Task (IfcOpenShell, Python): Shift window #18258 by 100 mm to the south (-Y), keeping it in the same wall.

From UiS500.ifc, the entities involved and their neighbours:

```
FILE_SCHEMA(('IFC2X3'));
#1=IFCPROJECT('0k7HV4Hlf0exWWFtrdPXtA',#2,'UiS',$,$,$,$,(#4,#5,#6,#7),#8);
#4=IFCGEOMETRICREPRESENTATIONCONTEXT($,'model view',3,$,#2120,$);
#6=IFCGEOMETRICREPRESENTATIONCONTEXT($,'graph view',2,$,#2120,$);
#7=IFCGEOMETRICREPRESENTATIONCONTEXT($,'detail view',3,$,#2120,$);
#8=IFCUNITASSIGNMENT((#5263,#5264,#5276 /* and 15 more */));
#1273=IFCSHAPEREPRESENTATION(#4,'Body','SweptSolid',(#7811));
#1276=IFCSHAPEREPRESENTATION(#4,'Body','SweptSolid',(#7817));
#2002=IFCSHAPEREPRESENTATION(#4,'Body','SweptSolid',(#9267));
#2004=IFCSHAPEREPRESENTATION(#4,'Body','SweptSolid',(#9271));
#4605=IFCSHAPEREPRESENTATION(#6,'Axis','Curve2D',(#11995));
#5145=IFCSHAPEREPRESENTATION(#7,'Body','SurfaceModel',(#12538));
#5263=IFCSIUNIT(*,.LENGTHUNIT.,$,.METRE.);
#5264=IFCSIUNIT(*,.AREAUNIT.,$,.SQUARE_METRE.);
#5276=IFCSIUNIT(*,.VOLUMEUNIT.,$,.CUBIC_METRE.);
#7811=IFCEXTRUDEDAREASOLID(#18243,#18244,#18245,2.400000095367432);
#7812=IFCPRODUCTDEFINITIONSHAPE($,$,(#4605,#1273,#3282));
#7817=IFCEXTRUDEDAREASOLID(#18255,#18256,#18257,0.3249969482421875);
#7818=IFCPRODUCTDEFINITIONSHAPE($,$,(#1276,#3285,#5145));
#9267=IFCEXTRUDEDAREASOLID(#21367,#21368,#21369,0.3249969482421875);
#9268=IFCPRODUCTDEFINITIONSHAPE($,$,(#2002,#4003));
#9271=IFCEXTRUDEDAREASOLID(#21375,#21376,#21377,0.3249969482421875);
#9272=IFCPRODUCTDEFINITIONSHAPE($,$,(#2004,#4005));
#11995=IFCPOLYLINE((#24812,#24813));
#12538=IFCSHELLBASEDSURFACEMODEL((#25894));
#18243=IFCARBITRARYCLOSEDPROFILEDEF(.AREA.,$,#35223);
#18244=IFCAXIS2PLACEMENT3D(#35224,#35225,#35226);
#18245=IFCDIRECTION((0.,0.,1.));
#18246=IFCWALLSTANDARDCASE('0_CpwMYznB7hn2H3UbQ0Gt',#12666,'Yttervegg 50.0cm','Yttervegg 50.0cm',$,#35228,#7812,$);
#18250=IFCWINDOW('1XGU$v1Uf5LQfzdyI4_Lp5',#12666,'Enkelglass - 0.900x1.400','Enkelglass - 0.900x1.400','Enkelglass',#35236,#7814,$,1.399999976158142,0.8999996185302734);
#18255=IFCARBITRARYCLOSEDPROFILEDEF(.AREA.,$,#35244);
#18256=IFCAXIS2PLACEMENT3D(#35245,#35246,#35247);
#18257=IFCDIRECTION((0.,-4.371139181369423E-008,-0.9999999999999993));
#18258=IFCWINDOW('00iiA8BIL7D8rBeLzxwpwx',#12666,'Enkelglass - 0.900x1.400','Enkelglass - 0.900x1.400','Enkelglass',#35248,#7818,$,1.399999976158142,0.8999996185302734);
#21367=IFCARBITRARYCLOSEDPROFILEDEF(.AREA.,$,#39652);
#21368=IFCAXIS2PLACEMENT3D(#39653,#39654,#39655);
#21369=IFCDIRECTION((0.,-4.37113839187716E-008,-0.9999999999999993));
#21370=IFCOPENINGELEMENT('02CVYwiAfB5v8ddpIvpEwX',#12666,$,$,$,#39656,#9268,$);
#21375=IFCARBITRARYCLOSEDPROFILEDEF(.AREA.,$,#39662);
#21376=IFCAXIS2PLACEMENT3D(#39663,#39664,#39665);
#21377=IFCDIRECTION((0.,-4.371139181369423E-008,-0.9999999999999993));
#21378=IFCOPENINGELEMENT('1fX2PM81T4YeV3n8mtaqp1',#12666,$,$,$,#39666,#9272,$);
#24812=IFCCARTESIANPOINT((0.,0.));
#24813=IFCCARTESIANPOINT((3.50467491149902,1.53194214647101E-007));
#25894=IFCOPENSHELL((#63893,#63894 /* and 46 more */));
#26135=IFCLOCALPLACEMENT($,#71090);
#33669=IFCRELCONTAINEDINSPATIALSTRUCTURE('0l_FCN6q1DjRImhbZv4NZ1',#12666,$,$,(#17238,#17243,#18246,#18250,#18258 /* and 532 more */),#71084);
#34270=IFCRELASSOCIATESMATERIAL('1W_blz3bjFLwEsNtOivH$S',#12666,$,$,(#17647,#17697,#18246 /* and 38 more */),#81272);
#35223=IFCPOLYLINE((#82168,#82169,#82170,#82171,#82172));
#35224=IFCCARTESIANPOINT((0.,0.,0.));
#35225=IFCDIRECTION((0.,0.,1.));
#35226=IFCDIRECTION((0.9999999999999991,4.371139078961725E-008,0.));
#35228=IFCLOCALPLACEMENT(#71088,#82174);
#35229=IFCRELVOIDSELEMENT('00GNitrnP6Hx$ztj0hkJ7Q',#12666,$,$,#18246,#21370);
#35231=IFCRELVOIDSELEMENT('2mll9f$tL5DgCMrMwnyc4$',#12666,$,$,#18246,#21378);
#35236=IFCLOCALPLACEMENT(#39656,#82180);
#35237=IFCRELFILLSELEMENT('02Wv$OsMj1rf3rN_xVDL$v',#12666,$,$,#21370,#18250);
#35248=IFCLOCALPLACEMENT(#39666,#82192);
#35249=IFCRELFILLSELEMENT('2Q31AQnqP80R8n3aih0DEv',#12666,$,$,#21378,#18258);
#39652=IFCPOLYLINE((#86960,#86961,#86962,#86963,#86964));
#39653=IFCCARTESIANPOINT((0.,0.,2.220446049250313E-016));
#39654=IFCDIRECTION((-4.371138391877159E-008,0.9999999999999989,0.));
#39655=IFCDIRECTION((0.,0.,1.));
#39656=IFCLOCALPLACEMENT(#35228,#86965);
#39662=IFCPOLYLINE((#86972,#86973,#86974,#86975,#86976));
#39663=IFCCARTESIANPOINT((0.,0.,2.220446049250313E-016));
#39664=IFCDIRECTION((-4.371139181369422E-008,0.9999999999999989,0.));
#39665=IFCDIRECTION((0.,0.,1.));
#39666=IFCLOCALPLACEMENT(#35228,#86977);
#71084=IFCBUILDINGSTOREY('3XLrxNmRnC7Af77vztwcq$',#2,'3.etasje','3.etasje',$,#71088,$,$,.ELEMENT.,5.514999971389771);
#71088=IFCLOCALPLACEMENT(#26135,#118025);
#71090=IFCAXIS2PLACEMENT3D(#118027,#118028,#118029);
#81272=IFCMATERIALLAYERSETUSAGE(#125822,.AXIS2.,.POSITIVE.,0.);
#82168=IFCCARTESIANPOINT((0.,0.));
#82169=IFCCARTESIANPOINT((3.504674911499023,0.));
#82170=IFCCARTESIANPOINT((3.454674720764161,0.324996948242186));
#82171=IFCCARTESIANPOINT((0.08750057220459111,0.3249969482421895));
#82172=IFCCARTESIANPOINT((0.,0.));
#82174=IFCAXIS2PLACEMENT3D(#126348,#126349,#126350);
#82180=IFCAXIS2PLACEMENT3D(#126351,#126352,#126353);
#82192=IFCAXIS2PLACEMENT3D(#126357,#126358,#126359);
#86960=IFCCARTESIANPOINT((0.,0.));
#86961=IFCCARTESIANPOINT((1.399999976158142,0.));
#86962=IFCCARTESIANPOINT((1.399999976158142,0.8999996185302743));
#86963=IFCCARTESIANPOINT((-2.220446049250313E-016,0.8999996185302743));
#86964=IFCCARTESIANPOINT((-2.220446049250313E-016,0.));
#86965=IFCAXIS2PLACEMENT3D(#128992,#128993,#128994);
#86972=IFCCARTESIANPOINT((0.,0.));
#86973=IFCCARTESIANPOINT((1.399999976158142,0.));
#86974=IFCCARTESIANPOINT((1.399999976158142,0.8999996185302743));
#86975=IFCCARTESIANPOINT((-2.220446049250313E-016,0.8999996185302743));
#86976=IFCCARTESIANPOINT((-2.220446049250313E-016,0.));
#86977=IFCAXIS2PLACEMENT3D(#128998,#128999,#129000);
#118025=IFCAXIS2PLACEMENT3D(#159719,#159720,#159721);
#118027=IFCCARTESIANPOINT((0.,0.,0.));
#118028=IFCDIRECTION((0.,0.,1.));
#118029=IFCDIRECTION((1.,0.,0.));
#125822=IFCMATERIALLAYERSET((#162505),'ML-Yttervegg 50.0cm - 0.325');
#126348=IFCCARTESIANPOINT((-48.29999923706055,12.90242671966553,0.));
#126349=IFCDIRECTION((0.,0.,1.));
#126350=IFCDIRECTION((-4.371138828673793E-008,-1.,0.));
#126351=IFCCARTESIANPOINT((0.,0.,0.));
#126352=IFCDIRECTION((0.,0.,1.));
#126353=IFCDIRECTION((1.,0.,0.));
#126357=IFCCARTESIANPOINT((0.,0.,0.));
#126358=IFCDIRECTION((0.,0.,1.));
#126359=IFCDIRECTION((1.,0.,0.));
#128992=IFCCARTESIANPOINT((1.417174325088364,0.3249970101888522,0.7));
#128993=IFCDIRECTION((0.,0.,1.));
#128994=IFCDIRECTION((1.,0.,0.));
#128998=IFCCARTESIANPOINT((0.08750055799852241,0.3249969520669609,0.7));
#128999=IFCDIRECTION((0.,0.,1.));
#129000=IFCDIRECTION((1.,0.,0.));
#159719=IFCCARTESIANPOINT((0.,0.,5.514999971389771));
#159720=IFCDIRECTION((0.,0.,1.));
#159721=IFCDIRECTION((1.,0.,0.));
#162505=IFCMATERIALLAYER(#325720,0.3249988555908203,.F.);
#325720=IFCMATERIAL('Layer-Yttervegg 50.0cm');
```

```python
import ifcopenshell
import ifcopenshell.api.geometry
import ifcopenshell.util.placement

model = ifcopenshell.open("UiS500.ifc")

window = model.by_guid("00iiA8BIL7D8rBeLzxwpwx")
opening = window.FillsVoids[0].RelatingOpeningElement
wall = opening.VoidsElements[0].RelatingBuildingElement

wall_matrix = ifcopenshell.util.placement.get_local_placement(wall.ObjectPlacement)
shift = wall_matrix[:3, 0] * 0.1
before = ifcopenshell.util.placement.get_local_placement(window.ObjectPlacement)[:3, 3].copy()

# The window is placed relative to its opening, so it follows when the opening moves.
matrix = ifcopenshell.util.placement.get_local_placement(opening.ObjectPlacement)
matrix[:3, 3] += shift
ifcopenshell.api.geometry.edit_object_placement(
    model, product=opening, matrix=matrix, is_si=False, should_transform_children=True
)

after = ifcopenshell.util.placement.get_local_placement(window.ObjectPlacement)[:3, 3]
print("window moved by", (after - before).round(3) + 0.0)

model.write("UiS500_edited.ifc")
```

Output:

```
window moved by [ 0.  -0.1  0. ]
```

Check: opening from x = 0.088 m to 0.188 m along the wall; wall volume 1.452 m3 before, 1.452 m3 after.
